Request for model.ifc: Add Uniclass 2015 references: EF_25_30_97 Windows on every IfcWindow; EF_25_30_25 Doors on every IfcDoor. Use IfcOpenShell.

First a look at what the model holds.

```python
import ifcopenshell

model = ifcopenshell.open("model.ifc")
print(model.schema)
print("classifications:", [c.Name for c in model.by_type("IfcClassification")])
for ifc_class in ("IfcDoor", "IfcRoof", "IfcStair", "IfcWall", "IfcWindow"):
    print(ifc_class, len(model.by_type(ifc_class)))
```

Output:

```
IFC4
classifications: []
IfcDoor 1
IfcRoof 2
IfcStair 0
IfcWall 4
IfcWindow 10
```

```python
import ifcopenshell
import ifcopenshell.api.classification

model = ifcopenshell.open("model.ifc")

system = ifcopenshell.api.classification.add_classification(model, classification="Uniclass 2015")

codes = {
    "IfcWindow": ("EF_25_30_97", "Windows"),
    "IfcDoor": ("EF_25_30_25", "Doors"),
}
for ifc_class, (code, name) in codes.items():
    products = model.by_type(ifc_class)
    ifcopenshell.api.classification.add_reference(
        model, products=products, classification=system, identification=code, name=name
    )
    print(code, len(products))

model.write("model_v2.ifc")
```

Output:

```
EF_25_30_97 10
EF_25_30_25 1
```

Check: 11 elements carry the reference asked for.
